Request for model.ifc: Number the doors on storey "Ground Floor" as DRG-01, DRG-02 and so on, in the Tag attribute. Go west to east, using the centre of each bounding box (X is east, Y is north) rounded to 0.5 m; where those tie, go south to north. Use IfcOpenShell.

First a look at what the model holds.

```python
import ifcopenshell
import ifcopenshell.util.element
import ifcopenshell.util.placement

model = ifcopenshell.open("model.ifc")
print(model.schema)
storey = next(s for s in model.by_type("IfcBuildingStorey") if s.Name == "Ground Floor")
doors = [e for e in ifcopenshell.util.element.get_decomposition(storey) if e.is_a("IfcDoor")]
for e in sorted(doors, key=lambda e: e.id()):
    origin = ifcopenshell.util.placement.get_local_placement(e.ObjectPlacement)[:3, 3]
    print(e.id(), e.Tag, e.Name, origin.round(2) + 0.0, sep=" | ")
```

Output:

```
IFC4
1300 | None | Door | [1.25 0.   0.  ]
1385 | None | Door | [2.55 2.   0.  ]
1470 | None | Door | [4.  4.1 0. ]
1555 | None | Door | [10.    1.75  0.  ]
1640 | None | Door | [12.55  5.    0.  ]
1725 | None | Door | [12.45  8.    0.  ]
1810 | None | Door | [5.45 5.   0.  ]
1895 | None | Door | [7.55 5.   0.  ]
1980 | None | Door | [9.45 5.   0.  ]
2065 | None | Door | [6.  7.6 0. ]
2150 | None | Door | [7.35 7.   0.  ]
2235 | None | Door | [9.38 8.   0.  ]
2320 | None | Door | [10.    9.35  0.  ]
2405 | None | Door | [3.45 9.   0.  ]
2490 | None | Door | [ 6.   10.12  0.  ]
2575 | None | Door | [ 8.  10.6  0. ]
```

```python
import ifcopenshell
import ifcopenshell.geom
import ifcopenshell.util.element
import ifcopenshell.util.shape

model = ifcopenshell.open("model.ifc")
settings = ifcopenshell.geom.settings()
settings.set("use-world-coords", True)


def centre(element):
    shape = ifcopenshell.geom.create_shape(settings, element)
    return ifcopenshell.util.shape.get_bbox_centroid(shape.geometry)


storey = next(s for s in model.by_type("IfcBuildingStorey") if s.Name == "Ground Floor")
doors = [e for e in ifcopenshell.util.element.get_decomposition(storey) if e.is_a("IfcDoor")]

# Insertion points can sit at a corner or the storey origin, so sort by the geometry (in metres).
centres = {e: centre(e) for e in doors}
doors.sort(key=lambda e: (round(centres[e][0] / 0.5), centres[e][1]))

for i, e in enumerate(doors, start=1):
    number = f"DRG-{i:02d}"
    e.Tag = number
    print(e.id(), number)

model.write("model-out.ifc")
```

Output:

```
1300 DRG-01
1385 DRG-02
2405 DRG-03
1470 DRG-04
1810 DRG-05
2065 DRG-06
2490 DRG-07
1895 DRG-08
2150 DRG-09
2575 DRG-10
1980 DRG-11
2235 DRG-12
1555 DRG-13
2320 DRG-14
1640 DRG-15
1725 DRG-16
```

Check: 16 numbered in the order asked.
